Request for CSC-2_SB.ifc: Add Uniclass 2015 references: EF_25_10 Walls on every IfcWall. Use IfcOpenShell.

First a look at what the model holds.

```python
import ifcopenshell

model = ifcopenshell.open("CSC-2_SB.ifc")
print(model.schema)
print("classifications:", [c.Name for c in model.by_type("IfcClassification")])
for ifc_class in ("IfcDoor", "IfcRoof", "IfcStair", "IfcWall", "IfcWindow"):
    print(ifc_class, len(model.by_type(ifc_class)))
```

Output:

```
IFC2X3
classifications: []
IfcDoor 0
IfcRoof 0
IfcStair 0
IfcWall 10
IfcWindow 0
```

```python
import ifcopenshell
import ifcopenshell.api.classification

model = ifcopenshell.open("CSC-2_SB.ifc")

# IFC2X3 requires Source and Edition and has no link from the project to the system.
system = model.create_entity("IfcClassification", Source="NBS", Edition="2015", Name="Uniclass 2015")

codes = {
    "IfcWall": ("EF_25_10", "Walls"),
}
for ifc_class, (code, name) in codes.items():
    products = model.by_type(ifc_class)
    ifcopenshell.api.classification.add_reference(
        model, products=products, classification=system, identification=code, name=name
    )
    print(code, len(products))

model.write("CSC-2_SB_rev.ifc")
```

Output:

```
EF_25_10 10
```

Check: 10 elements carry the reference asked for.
